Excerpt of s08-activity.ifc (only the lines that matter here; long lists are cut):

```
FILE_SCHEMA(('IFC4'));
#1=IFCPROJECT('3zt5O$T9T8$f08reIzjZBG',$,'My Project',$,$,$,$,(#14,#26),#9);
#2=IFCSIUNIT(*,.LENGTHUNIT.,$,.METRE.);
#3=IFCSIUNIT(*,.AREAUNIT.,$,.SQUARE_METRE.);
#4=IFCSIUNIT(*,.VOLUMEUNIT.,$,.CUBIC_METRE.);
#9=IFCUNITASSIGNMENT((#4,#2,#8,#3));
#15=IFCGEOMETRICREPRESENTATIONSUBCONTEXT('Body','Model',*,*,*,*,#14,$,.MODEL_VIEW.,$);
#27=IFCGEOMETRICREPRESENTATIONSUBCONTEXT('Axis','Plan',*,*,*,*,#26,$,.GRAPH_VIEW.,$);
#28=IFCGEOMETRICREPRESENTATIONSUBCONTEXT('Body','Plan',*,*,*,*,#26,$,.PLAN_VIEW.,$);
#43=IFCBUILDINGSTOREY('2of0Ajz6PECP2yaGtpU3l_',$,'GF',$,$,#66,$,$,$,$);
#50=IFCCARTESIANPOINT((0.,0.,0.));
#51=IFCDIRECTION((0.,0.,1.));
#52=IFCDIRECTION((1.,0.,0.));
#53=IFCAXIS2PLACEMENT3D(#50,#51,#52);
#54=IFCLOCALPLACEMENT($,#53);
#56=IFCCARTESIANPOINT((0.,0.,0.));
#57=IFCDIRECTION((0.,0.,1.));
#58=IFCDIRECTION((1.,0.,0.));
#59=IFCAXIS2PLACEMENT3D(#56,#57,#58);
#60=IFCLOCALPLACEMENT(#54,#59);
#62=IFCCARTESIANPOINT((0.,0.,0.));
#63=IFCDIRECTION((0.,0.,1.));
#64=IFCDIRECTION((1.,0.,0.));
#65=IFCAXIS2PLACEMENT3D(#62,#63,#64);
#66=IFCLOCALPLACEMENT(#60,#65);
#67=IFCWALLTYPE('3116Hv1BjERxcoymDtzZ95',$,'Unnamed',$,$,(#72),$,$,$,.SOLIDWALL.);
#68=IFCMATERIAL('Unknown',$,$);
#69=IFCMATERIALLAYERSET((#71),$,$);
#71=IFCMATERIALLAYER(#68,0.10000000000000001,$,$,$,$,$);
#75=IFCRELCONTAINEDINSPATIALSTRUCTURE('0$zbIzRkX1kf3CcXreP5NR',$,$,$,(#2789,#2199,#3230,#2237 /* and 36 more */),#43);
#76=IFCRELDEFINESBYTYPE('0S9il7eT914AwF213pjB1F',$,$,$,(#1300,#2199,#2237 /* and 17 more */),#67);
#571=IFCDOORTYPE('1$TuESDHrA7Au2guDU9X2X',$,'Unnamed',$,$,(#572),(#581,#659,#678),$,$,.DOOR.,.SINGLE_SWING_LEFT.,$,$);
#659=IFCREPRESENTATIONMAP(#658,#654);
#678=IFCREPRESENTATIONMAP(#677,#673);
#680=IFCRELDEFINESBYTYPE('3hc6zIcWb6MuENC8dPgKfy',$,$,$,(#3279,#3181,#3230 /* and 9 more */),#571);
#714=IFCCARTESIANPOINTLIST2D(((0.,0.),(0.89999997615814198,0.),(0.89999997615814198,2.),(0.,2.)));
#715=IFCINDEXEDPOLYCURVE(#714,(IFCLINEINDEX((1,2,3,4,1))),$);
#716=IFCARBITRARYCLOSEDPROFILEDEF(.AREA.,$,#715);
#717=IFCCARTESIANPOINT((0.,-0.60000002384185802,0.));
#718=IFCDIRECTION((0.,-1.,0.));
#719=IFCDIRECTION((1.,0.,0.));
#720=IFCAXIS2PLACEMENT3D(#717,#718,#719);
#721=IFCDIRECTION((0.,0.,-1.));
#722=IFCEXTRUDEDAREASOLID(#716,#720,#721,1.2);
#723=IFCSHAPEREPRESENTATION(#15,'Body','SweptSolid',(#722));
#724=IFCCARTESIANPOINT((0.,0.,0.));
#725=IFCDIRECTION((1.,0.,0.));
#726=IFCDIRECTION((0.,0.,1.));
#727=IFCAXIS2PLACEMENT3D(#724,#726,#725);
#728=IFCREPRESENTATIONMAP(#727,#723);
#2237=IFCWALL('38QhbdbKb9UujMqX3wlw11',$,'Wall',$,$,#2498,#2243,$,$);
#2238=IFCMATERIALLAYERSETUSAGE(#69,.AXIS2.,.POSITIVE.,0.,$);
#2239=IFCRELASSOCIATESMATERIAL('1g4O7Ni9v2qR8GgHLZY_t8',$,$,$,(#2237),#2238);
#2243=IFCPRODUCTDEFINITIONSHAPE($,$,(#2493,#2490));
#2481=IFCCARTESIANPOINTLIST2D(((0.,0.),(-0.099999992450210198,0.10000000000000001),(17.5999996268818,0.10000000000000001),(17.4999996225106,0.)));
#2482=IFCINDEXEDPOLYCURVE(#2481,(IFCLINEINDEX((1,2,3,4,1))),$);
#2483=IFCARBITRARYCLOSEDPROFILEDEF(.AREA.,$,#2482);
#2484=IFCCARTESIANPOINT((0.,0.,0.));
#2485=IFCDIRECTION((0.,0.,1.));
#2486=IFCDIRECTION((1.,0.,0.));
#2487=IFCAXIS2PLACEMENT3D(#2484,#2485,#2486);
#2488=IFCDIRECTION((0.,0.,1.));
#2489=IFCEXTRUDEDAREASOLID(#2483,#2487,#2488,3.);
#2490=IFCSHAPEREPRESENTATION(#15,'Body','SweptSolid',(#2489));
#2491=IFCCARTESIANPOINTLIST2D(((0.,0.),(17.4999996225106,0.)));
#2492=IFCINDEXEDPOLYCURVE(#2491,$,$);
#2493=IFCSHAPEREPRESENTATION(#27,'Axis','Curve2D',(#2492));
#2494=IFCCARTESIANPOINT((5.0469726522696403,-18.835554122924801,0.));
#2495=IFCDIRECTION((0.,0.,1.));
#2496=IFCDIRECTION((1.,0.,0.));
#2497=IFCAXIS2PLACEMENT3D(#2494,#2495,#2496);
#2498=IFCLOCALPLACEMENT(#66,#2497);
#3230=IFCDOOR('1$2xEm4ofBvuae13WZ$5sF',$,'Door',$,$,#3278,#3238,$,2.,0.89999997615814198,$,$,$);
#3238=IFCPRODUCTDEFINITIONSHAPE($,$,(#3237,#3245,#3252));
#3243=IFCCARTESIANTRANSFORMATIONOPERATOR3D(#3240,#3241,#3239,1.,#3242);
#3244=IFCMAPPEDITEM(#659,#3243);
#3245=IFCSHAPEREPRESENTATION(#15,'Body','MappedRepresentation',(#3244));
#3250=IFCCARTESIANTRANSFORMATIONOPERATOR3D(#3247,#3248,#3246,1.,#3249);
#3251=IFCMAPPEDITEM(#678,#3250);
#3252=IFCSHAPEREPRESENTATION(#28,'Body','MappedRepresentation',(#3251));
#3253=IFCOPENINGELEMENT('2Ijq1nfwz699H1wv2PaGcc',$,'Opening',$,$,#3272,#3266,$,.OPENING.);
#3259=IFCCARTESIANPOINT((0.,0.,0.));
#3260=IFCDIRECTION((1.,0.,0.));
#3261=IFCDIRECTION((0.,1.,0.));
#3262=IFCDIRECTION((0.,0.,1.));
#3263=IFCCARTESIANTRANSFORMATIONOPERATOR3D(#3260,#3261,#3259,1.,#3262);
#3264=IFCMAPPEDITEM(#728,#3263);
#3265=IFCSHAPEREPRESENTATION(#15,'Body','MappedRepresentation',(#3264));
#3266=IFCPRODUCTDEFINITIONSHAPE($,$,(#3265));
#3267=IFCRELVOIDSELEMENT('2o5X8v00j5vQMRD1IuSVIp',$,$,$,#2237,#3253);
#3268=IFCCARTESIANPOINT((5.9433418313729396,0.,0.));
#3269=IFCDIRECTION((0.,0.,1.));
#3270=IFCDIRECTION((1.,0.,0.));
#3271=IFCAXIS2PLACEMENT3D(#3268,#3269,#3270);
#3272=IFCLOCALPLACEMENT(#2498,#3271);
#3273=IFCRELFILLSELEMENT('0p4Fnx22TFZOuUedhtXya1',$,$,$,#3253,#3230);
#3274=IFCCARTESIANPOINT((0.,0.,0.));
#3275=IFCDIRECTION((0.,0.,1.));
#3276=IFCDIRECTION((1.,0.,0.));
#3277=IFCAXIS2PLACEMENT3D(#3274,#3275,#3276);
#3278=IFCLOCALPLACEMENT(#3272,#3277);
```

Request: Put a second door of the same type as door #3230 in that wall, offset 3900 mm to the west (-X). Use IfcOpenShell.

```python
import ifcopenshell
import ifcopenshell.api.feature
import ifcopenshell.api.geometry
import ifcopenshell.api.root
import ifcopenshell.geom
import ifcopenshell.util.element
import ifcopenshell.util.placement
import ifcopenshell.util.shape
import ifcopenshell.util.unit

model = ifcopenshell.open("s08-activity.ifc")
unit_scale = ifcopenshell.util.unit.calculate_unit_scale(model)
settings = ifcopenshell.geom.settings()


def volume(element):
    """Net volume in cubic metres, openings subtracted."""
    shape = ifcopenshell.geom.create_shape(settings, element)
    return ifcopenshell.util.shape.get_volume(shape.geometry)


door = model.by_guid("1$2xEm4ofBvuae13WZ$5sF")
opening = door.FillsVoids[0].RelatingOpeningElement
wall = opening.VoidsElements[0].RelatingBuildingElement
before = volume(wall)
shift = ifcopenshell.util.placement.get_local_placement(wall.ObjectPlacement)[:3, 0] * -3.9 / unit_scale

# copy_class copies the void relationship, type, container and properties, but no geometry.
new_opening = ifcopenshell.api.root.copy_class(model, product=opening)
new_opening.Representation = ifcopenshell.util.element.copy_deep(
    model, opening.Representation, exclude=["IfcGeometricRepresentationContext", "IfcRepresentationMap"]
)
new_door = ifcopenshell.api.root.copy_class(model, product=door)
new_door.Representation = ifcopenshell.util.element.copy_deep(
    model, door.Representation, exclude=["IfcGeometricRepresentationContext", "IfcRepresentationMap"]
)
ifcopenshell.api.feature.add_filling(model, opening=new_opening, element=new_door)

for old, new in ((opening, new_opening), (door, new_door)):
    matrix = ifcopenshell.util.placement.get_local_placement(old.ObjectPlacement)
    matrix[:3, 3] += shift
    ifcopenshell.api.geometry.edit_object_placement(model, product=new, matrix=matrix, is_si=False)

after = volume(wall)

print(f"wall volume {before:.3f} -> {after:.3f} m3")

model.write("s08-activity_updated.ifc")
```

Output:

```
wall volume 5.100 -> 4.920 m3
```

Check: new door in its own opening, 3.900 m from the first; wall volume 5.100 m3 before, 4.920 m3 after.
